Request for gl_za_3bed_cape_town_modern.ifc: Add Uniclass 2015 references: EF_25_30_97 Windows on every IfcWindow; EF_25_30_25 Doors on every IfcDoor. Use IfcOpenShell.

First a look at what the model holds.

```python
import ifcopenshell

model = ifcopenshell.open("gl_za_3bed_cape_town_modern.ifc")
print(model.schema)
print("classifications:", [c.Name for c in model.by_type("IfcClassification")])
for ifc_class in ("IfcDoor", "IfcRoof", "IfcStair", "IfcWall", "IfcWindow"):
    print(ifc_class, len(model.by_type(ifc_class)))
```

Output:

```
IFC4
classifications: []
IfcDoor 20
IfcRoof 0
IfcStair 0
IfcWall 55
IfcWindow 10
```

```python
import ifcopenshell
import ifcopenshell.api.classification

model = ifcopenshell.open("gl_za_3bed_cape_town_modern.ifc")

system = ifcopenshell.api.classification.add_classification(model, classification="Uniclass 2015")

codes = {
    "IfcWindow": ("EF_25_30_97", "Windows"),
    "IfcDoor": ("EF_25_30_25", "Doors"),
}
for ifc_class, (code, name) in codes.items():
    products = model.by_type(ifc_class)
    ifcopenshell.api.classification.add_reference(
        model, products=products, classification=system, identification=code, name=name
    )
    print(code, len(products))

model.write("gl_za_3bed_cape_town_modern_rev.ifc")
```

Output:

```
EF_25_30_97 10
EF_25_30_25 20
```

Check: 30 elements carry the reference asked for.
